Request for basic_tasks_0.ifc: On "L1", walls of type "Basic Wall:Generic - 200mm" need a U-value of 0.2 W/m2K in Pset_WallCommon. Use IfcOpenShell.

First a look at what the model holds.

```python
import ifcopenshell
import ifcopenshell.util.element

model = ifcopenshell.open("basic_tasks_0.ifc")
print(model.schema)
storey = next(s for s in model.by_type("IfcBuildingStorey") if s.Name == "L1")
walls = [e for e in ifcopenshell.util.element.get_decomposition(storey) if e.is_a("IfcWall")]
seen = {}
for e in walls:
    element_type = ifcopenshell.util.element.get_type(e)
    key = (element_type.Name if element_type != e and element_type else None, ifcopenshell.util.element.get_pset(e, "Pset_WallCommon", "ThermalTransmittance"))
    seen[key] = seen.get(key, 0) + 1
for (name, value), count in sorted(seen.items(), key=str):
    print(count, "x", name, "|", value)
```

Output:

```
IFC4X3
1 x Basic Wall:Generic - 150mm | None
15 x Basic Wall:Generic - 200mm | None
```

```python
import ifcopenshell
import ifcopenshell.api.pset
import ifcopenshell.util.element

model = ifcopenshell.open("basic_tasks_0.ifc")

storey = next(s for s in model.by_type("IfcBuildingStorey") if s.Name == "L1")
walls = [e for e in ifcopenshell.util.element.get_decomposition(storey) if e.is_a("IfcWall")]

count = 0
for e in walls:
    element_type = ifcopenshell.util.element.get_type(e)
    if element_type in (None, e) or element_type.Name != "Basic Wall:Generic - 200mm":
        continue
    # add_pset returns the element's existing set when there is one.
    pset = ifcopenshell.api.pset.add_pset(model, product=e, name="Pset_WallCommon")
    ifcopenshell.api.pset.edit_pset(model, pset=pset, properties={"ThermalTransmittance": 0.2})
    count += 1

print(count, "walls updated")

model.write("basic_tasks_0_edited.ifc")
```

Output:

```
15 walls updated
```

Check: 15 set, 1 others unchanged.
